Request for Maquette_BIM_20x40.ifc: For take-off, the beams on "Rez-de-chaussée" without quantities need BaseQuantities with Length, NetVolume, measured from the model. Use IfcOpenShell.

First a look at what the model holds.

```python
import ifcopenshell
import ifcopenshell.util.element
import ifcopenshell.util.unit

model = ifcopenshell.open("Maquette_BIM_20x40.ifc")
print(model.schema)
for unit_type in ("LENGTHUNIT", "AREAUNIT", "VOLUMEUNIT"):
    print(unit_type, ifcopenshell.util.unit.calculate_unit_scale(model, unit_type))
storey = next(s for s in model.by_type("IfcBuildingStorey") if s.Name == "Rez-de-chaussée")
beams = [e for e in ifcopenshell.util.element.get_decomposition(storey) if e.is_a("IfcBeam")]
for e in sorted(beams, key=lambda e: e.id()):
    print(e.id(), e.is_a(), e.Name, list(ifcopenshell.util.element.get_psets(e, qtos_only=True)), sep=" | ")
```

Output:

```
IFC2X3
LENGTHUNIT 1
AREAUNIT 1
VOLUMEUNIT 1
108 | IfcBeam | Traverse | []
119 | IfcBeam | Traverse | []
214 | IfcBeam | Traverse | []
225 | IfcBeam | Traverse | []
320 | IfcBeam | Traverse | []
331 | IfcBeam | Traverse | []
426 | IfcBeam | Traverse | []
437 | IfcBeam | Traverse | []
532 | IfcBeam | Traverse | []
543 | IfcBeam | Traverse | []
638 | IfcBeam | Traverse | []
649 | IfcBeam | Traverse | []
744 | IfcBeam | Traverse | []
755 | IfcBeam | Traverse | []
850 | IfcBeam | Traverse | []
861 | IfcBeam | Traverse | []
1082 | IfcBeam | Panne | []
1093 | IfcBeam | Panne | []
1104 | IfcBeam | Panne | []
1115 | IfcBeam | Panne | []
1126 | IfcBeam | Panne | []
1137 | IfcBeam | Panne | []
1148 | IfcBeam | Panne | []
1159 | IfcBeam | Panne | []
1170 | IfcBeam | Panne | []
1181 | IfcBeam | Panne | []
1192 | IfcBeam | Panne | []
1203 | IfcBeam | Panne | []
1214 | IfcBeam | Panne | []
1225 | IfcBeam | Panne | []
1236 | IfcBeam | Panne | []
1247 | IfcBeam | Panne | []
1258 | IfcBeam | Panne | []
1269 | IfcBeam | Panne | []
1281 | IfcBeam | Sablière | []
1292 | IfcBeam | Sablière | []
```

```python
import ifcopenshell
import ifcopenshell.api.pset
import ifcopenshell.geom
import ifcopenshell.util.element
import ifcopenshell.util.shape
import ifcopenshell.util.unit

model = ifcopenshell.open("Maquette_BIM_20x40.ifc")
unit_scale = ifcopenshell.util.unit.calculate_unit_scale(model)
volume_scale = ifcopenshell.util.unit.calculate_unit_scale(model, "VOLUMEUNIT")
settings = ifcopenshell.geom.settings()

storey = next(s for s in model.by_type("IfcBuildingStorey") if s.Name == "Rez-de-chaussée")
beams = [e for e in ifcopenshell.util.element.get_decomposition(storey) if e.is_a("IfcBeam")]

for e in sorted(beams, key=lambda e: e.id()):
    if ifcopenshell.util.element.get_psets(e, qtos_only=True, should_inherit=False):
        continue
    # Geometry comes back in metres, in the element's own axes.
    shape = ifcopenshell.geom.create_shape(settings, e)
    values = {
        "Length": ifcopenshell.util.shape.get_max_xyz(shape.geometry) / unit_scale,
        "NetVolume": ifcopenshell.util.shape.get_volume(shape.geometry) / volume_scale,
    }
    qto = ifcopenshell.api.pset.add_qto(model, product=e, name="BaseQuantities")
    ifcopenshell.api.pset.edit_qto(model, qto=qto, properties=values)
    print(e.id(), {k: round(v, 3) for k, v in values.items()})

model.write("Maquette_BIM_20x40_edited.ifc")
```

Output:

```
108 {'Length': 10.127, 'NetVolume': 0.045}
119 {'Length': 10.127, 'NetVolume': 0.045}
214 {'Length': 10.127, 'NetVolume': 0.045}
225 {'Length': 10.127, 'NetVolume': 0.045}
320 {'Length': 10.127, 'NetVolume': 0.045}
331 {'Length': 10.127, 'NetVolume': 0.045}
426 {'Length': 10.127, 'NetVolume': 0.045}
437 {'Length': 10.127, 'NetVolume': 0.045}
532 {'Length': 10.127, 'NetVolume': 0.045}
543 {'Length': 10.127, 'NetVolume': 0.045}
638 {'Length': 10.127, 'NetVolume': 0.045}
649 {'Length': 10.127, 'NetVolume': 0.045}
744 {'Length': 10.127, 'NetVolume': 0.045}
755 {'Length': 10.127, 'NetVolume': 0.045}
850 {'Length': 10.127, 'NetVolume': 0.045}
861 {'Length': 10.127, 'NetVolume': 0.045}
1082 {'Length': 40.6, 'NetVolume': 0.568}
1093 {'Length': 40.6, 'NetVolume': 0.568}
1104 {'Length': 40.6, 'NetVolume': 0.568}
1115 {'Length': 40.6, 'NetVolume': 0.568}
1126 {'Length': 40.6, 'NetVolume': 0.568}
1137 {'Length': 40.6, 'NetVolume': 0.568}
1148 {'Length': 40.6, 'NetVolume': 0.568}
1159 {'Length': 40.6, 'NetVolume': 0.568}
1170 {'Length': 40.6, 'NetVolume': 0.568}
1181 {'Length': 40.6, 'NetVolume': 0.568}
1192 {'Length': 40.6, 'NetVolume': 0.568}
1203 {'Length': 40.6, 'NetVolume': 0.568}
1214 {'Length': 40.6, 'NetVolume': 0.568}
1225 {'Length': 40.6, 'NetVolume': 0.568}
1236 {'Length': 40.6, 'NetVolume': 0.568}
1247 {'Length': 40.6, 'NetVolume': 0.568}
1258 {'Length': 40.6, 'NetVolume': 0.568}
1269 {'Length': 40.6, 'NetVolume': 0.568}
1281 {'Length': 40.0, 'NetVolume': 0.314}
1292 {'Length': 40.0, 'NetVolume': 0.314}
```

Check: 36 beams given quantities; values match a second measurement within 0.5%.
